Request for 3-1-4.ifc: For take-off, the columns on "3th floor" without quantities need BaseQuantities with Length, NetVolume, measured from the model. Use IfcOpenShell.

First a look at what the model holds.

```python
import ifcopenshell
import ifcopenshell.util.element
import ifcopenshell.util.unit

model = ifcopenshell.open("3-1-4.ifc")
print(model.schema)
for unit_type in ("LENGTHUNIT", "AREAUNIT", "VOLUMEUNIT"):
    print(unit_type, ifcopenshell.util.unit.calculate_unit_scale(model, unit_type))
storey = next(s for s in model.by_type("IfcBuildingStorey") if s.Name == "3th floor")
columns = [e for e in ifcopenshell.util.element.get_decomposition(storey) if e.is_a("IfcColumn")]
for e in sorted(columns, key=lambda e: e.id()):
    print(e.id(), e.is_a(), e.Name, list(ifcopenshell.util.element.get_psets(e, qtos_only=True)), sep=" | ")
```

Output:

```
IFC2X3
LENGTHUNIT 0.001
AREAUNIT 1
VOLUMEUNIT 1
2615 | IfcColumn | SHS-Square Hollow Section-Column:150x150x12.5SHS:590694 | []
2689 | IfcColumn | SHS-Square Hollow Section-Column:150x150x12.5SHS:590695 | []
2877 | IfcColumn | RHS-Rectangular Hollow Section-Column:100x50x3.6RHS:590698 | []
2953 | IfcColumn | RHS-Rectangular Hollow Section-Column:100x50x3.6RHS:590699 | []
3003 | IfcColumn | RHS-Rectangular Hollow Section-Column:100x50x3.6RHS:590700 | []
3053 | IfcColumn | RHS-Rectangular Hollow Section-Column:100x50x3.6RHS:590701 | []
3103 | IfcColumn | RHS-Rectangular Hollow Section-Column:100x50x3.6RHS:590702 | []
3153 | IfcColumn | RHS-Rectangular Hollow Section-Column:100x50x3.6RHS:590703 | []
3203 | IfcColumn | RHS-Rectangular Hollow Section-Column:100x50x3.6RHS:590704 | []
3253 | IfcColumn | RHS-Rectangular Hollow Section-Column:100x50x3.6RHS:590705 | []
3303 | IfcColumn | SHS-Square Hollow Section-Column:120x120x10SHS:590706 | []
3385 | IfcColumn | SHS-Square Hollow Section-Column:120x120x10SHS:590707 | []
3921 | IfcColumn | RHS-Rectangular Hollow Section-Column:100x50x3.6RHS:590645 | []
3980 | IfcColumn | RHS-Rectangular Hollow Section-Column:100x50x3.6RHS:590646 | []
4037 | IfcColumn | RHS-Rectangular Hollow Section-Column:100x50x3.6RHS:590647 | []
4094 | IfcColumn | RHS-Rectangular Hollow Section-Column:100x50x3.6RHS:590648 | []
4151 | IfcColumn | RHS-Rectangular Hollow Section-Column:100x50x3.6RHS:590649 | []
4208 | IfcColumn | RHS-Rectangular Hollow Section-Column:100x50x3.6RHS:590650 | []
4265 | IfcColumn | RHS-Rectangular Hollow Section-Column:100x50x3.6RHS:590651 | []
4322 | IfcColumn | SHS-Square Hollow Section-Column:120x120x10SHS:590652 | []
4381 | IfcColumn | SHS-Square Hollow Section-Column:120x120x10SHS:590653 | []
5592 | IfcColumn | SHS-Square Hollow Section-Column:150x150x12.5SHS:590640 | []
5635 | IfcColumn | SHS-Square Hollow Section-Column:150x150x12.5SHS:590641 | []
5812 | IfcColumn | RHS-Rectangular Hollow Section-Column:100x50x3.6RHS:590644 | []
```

```python
import ifcopenshell
import ifcopenshell.api.pset
import ifcopenshell.geom
import ifcopenshell.util.element
import ifcopenshell.util.shape
import ifcopenshell.util.unit

model = ifcopenshell.open("3-1-4.ifc")
unit_scale = ifcopenshell.util.unit.calculate_unit_scale(model)
volume_scale = ifcopenshell.util.unit.calculate_unit_scale(model, "VOLUMEUNIT")
settings = ifcopenshell.geom.settings()

storey = next(s for s in model.by_type("IfcBuildingStorey") if s.Name == "3th floor")
columns = [e for e in ifcopenshell.util.element.get_decomposition(storey) if e.is_a("IfcColumn")]

for e in sorted(columns, key=lambda e: e.id()):
    if ifcopenshell.util.element.get_psets(e, qtos_only=True, should_inherit=False):
        continue
    # Geometry comes back in metres, in the element's own axes.
    shape = ifcopenshell.geom.create_shape(settings, e)
    values = {
        "Length": ifcopenshell.util.shape.get_z(shape.geometry) / unit_scale,
        "NetVolume": ifcopenshell.util.shape.get_volume(shape.geometry) / volume_scale,
    }
    qto = ifcopenshell.api.pset.add_qto(model, product=e, name="BaseQuantities")
    ifcopenshell.api.pset.edit_qto(model, qto=qto, properties=values)
    print(e.id(), {k: round(v, 3) for k, v in values.items()})

model.write("3-1-4_updated.ifc")
```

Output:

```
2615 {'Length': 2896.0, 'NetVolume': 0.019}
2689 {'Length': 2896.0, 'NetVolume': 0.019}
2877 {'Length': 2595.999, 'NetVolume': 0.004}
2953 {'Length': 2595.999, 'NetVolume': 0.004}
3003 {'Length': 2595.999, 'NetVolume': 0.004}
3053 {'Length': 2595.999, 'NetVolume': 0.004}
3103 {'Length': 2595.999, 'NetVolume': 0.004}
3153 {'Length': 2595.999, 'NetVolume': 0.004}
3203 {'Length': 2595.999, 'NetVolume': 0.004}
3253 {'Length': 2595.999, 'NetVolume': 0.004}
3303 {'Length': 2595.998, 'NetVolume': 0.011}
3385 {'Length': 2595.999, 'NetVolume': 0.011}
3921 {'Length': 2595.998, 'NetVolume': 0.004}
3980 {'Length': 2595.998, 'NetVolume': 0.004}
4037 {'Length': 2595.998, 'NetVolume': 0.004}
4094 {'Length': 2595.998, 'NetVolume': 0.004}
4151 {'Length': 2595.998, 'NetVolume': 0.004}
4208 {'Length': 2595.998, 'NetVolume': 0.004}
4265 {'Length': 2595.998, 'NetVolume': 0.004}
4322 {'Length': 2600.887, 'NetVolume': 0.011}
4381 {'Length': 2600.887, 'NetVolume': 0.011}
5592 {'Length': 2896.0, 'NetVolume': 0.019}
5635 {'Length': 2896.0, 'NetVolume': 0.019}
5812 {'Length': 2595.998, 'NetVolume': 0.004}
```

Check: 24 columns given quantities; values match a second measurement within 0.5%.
